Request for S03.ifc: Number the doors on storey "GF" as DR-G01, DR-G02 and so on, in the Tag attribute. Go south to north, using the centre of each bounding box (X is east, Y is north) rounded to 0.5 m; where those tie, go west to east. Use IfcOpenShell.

First a look at what the model holds.

```python
import ifcopenshell
import ifcopenshell.util.element
import ifcopenshell.util.placement

model = ifcopenshell.open("S03.ifc")
print(model.schema)
storey = next(s for s in model.by_type("IfcBuildingStorey") if s.Name == "GF")
doors = [e for e in ifcopenshell.util.element.get_decomposition(storey) if e.is_a("IfcDoor")]
for e in sorted(doors, key=lambda e: e.id()):
    origin = ifcopenshell.util.placement.get_local_placement(e.ObjectPlacement)[:3, 3]
    print(e.id(), e.Tag, e.Name, origin.round(2) + 0.0, sep=" | ")
```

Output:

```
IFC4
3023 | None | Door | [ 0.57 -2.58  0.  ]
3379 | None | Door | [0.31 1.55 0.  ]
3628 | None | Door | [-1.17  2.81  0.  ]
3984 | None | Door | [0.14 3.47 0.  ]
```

```python
import ifcopenshell
import ifcopenshell.geom
import ifcopenshell.util.element
import ifcopenshell.util.shape

model = ifcopenshell.open("S03.ifc")
settings = ifcopenshell.geom.settings()
settings.set("use-world-coords", True)


def centre(element):
    shape = ifcopenshell.geom.create_shape(settings, element)
    return ifcopenshell.util.shape.get_bbox_centroid(shape.geometry)


storey = next(s for s in model.by_type("IfcBuildingStorey") if s.Name == "GF")
doors = [e for e in ifcopenshell.util.element.get_decomposition(storey) if e.is_a("IfcDoor")]

# Insertion points can sit at a corner or the storey origin, so sort by the geometry (in metres).
centres = {e: centre(e) for e in doors}
doors.sort(key=lambda e: (round(centres[e][1] / 0.5), centres[e][0]))

for i, e in enumerate(doors, start=1):
    number = f"DR-G{i:02d}"
    e.Tag = number
    print(e.id(), number)

model.write("S03_edited.ifc")
```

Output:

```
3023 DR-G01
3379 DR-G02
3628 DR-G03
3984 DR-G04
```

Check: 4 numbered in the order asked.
